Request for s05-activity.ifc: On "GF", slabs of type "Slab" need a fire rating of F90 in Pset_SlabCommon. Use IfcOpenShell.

First a look at what the model holds.

```python
import ifcopenshell
import ifcopenshell.util.element

model = ifcopenshell.open("s05-activity.ifc")
print(model.schema)
storey = next(s for s in model.by_type("IfcBuildingStorey") if s.Name == "GF")
slabs = [e for e in ifcopenshell.util.element.get_decomposition(storey) if e.is_a("IfcSlab")]
seen = {}
for e in slabs:
    element_type = ifcopenshell.util.element.get_type(e)
    key = (element_type.Name if element_type != e and element_type else None, ifcopenshell.util.element.get_pset(e, "Pset_SlabCommon", "FireRating"))
    seen[key] = seen.get(key, 0) + 1
for (name, value), count in sorted(seen.items(), key=str):
    print(count, "x", name, "|", value)
```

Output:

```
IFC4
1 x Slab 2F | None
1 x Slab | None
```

```python
import ifcopenshell
import ifcopenshell.api.pset
import ifcopenshell.util.element

model = ifcopenshell.open("s05-activity.ifc")

storey = next(s for s in model.by_type("IfcBuildingStorey") if s.Name == "GF")
slabs = [e for e in ifcopenshell.util.element.get_decomposition(storey) if e.is_a("IfcSlab")]

count = 0
for e in slabs:
    element_type = ifcopenshell.util.element.get_type(e)
    if element_type in (None, e) or element_type.Name != "Slab":
        continue
    # add_pset returns the element's existing set when there is one.
    pset = ifcopenshell.api.pset.add_pset(model, product=e, name="Pset_SlabCommon")
    ifcopenshell.api.pset.edit_pset(model, pset=pset, properties={"FireRating": "F90"})
    count += 1

print(count, "slabs updated")

model.write("s05-activity_edited.ifc")
```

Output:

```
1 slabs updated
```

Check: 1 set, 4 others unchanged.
